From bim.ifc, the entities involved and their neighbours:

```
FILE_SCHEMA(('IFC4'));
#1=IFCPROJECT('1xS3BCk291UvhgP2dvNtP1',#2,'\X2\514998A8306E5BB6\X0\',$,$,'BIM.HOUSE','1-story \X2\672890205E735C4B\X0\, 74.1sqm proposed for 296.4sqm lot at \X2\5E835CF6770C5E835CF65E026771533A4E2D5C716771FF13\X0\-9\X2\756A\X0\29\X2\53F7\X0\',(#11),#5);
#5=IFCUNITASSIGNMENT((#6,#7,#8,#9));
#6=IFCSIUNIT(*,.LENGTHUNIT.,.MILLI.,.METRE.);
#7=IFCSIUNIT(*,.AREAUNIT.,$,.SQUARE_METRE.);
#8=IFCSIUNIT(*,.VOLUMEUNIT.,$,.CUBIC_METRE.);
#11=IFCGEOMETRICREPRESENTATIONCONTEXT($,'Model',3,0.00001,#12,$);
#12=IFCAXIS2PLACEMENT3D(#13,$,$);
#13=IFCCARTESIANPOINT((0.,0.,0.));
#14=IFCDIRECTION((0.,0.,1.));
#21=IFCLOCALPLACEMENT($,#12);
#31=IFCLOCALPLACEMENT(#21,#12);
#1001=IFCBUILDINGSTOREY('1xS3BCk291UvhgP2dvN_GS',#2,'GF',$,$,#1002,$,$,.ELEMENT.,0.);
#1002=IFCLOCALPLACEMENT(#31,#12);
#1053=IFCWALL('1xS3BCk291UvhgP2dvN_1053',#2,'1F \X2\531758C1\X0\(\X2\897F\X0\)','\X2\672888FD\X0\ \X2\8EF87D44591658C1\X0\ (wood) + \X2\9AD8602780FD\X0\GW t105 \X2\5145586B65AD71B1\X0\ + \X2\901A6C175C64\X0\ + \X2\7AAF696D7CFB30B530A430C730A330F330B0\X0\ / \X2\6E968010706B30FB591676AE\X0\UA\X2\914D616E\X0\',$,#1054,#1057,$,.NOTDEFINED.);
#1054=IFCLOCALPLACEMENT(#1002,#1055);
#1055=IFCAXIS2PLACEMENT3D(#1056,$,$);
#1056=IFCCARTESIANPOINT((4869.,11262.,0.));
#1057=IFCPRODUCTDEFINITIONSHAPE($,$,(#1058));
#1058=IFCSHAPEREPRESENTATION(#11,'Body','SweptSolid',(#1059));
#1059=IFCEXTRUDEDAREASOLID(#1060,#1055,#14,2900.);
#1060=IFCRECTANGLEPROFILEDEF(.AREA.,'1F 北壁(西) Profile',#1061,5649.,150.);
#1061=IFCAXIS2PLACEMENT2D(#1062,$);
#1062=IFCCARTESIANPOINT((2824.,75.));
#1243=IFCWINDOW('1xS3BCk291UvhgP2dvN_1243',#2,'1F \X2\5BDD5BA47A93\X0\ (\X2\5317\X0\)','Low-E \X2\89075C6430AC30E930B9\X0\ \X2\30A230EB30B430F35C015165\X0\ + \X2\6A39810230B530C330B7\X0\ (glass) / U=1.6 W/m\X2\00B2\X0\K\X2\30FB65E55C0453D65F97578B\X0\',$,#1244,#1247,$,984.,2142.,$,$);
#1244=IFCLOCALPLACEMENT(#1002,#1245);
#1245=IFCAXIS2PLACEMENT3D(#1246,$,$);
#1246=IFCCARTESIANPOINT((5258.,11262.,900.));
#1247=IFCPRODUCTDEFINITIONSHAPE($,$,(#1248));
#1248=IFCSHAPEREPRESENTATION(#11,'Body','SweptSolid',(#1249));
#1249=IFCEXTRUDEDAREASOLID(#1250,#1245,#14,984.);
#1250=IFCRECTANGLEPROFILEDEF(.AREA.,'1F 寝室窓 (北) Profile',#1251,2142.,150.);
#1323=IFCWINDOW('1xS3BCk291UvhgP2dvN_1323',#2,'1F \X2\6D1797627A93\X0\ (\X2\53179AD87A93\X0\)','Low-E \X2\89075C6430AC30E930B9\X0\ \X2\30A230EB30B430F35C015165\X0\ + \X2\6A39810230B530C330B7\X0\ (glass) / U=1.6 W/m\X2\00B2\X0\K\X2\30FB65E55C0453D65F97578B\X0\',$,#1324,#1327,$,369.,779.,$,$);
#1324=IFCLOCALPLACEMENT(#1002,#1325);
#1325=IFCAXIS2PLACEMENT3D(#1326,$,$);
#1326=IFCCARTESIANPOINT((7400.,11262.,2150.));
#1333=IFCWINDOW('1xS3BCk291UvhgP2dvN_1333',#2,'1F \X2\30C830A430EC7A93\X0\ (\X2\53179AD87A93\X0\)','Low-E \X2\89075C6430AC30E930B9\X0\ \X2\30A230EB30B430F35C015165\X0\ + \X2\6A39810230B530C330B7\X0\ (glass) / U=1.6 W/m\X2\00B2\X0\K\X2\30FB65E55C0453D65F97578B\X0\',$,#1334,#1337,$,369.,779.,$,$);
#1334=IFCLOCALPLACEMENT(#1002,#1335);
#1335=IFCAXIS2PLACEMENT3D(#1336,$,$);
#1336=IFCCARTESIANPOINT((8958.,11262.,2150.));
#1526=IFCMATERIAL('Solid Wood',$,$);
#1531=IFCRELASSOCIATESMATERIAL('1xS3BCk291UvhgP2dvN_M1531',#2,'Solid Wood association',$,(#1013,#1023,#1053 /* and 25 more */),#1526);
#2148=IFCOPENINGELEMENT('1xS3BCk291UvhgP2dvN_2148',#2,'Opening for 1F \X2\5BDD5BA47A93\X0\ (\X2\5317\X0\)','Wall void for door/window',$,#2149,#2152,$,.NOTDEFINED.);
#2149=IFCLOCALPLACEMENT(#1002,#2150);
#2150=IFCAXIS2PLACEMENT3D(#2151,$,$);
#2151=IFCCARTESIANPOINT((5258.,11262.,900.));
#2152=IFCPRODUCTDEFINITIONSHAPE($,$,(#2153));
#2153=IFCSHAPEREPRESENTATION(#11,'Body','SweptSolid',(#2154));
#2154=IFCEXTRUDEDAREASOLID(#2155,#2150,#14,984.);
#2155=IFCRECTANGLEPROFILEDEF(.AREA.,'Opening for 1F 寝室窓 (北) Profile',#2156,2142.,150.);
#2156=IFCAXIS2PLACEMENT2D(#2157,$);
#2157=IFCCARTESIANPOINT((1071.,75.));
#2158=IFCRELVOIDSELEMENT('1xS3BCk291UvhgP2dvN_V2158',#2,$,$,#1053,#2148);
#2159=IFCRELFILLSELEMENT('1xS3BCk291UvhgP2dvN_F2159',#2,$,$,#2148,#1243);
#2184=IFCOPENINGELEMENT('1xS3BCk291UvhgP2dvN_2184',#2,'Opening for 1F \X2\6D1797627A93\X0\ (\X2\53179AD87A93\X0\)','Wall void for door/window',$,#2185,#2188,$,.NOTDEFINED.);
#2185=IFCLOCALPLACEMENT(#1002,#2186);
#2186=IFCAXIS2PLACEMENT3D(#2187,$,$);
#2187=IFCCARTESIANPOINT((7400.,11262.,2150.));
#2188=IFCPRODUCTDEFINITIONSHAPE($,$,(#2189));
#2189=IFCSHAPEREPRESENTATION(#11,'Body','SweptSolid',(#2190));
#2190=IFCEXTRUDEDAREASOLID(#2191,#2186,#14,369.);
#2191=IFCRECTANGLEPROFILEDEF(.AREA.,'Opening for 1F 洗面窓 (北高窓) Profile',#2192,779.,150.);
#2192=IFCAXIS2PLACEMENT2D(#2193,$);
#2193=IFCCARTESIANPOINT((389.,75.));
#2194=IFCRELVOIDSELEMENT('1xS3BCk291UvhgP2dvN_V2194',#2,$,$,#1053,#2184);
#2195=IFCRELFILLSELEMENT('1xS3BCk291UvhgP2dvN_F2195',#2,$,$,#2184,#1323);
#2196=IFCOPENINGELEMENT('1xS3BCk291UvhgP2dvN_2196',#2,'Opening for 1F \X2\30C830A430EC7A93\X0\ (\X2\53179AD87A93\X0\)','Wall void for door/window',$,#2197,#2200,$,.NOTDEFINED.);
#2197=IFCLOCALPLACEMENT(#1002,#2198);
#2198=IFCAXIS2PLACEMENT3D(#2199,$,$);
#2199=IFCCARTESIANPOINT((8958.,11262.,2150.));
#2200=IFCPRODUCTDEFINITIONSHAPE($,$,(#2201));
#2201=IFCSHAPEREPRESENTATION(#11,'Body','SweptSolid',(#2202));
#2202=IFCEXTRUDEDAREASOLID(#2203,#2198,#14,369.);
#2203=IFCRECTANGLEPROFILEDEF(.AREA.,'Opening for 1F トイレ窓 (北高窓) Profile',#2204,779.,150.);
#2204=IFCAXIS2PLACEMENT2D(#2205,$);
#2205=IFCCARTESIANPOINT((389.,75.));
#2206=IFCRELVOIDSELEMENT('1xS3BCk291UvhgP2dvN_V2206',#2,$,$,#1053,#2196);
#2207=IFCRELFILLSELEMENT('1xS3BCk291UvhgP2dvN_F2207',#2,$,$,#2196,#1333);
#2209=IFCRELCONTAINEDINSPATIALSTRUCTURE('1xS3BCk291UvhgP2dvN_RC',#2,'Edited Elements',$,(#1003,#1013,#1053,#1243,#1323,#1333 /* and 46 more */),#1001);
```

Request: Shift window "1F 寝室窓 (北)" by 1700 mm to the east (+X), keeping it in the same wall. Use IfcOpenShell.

```python
import ifcopenshell
import ifcopenshell.api.geometry
import ifcopenshell.util.placement
import ifcopenshell.util.unit

model = ifcopenshell.open("bim.ifc")
unit_scale = ifcopenshell.util.unit.calculate_unit_scale(model)

window = model.by_guid("1xS3BCk291UvhgP2dvN_1243")
opening = window.FillsVoids[0].RelatingOpeningElement
wall = opening.VoidsElements[0].RelatingBuildingElement

wall_matrix = ifcopenshell.util.placement.get_local_placement(wall.ObjectPlacement)
shift = wall_matrix[:3, 0] * 1.7 / unit_scale
before = ifcopenshell.util.placement.get_local_placement(window.ObjectPlacement)[:3, 3].copy()

# The window is not placed relative to its opening, so move both.
for product in (opening, window):
    matrix = ifcopenshell.util.placement.get_local_placement(product.ObjectPlacement)
    matrix[:3, 3] += shift
    ifcopenshell.api.geometry.edit_object_placement(model, product=product, matrix=matrix, is_si=False)

after = ifcopenshell.util.placement.get_local_placement(window.ObjectPlacement)[:3, 3]
print("window moved by", (after - before).round(3) + 0.0)

model.write("bim_updated.ifc")
```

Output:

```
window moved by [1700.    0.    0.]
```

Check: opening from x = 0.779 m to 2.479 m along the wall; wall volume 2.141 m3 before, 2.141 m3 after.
